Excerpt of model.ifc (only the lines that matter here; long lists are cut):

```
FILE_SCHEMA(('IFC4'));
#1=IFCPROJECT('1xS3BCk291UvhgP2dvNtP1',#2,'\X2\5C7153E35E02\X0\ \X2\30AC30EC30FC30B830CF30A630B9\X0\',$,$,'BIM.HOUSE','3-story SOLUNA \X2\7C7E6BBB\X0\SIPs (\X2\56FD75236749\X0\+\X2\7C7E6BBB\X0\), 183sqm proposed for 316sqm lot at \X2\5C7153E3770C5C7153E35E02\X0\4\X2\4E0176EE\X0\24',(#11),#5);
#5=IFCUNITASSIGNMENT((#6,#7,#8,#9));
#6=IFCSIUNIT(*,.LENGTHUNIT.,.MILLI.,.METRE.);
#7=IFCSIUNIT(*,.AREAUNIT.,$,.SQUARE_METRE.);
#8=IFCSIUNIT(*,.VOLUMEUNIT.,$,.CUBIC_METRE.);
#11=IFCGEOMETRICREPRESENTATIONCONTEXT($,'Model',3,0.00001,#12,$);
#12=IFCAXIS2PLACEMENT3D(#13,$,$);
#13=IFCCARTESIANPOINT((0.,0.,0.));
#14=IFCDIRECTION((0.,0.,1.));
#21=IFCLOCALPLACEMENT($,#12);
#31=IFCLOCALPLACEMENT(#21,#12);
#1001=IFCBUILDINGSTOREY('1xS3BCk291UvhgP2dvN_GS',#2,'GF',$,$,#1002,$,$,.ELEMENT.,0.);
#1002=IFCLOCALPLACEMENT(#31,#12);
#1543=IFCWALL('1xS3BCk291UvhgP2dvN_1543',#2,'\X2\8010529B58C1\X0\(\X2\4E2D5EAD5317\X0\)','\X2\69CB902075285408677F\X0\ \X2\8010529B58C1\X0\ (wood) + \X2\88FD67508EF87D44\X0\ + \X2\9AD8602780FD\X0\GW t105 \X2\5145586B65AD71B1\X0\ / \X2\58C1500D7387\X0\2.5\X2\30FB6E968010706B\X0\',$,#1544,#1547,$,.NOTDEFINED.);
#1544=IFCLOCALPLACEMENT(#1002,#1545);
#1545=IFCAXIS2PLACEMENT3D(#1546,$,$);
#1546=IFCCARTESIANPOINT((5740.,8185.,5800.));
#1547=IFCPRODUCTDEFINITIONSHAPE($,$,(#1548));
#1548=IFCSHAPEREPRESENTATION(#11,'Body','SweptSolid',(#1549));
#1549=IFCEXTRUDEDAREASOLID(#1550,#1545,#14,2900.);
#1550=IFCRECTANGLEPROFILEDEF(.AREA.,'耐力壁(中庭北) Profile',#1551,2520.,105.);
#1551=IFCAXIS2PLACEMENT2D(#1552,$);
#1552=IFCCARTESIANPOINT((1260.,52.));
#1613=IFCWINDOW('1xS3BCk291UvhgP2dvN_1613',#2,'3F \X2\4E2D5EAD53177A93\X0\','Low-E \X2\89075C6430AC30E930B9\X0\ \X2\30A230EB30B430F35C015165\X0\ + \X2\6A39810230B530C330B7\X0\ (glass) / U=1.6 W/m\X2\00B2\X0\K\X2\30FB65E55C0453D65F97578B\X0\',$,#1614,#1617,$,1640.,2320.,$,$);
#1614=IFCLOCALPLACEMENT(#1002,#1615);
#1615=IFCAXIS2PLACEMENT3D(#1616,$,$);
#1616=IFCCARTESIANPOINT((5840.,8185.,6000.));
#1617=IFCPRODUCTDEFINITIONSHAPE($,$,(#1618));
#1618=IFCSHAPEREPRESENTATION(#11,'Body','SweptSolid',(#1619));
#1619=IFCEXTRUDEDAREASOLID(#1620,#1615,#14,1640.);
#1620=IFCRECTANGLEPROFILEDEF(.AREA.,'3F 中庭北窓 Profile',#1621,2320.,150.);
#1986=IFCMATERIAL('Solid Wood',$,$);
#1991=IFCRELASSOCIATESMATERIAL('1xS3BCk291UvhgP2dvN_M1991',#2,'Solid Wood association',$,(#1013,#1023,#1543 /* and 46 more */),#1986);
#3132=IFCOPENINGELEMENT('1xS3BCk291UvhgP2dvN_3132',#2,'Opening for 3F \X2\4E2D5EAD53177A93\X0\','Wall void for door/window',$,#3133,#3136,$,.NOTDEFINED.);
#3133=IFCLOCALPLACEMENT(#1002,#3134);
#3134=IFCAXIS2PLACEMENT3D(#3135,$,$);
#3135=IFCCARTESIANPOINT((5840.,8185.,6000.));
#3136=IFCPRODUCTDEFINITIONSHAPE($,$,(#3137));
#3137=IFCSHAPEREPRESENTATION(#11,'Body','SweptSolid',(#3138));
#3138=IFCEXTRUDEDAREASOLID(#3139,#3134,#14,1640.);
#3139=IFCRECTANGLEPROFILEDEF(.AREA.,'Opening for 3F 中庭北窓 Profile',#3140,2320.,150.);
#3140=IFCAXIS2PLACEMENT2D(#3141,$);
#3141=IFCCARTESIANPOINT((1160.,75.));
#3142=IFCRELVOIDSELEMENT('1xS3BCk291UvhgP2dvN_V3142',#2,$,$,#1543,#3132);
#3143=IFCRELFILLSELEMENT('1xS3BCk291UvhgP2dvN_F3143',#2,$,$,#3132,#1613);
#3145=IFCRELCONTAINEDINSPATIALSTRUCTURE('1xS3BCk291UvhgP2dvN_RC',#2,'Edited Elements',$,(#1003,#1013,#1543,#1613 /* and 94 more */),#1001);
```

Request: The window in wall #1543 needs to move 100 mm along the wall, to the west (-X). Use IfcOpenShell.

```python
import ifcopenshell
import ifcopenshell.api.geometry
import ifcopenshell.util.placement
import ifcopenshell.util.unit

model = ifcopenshell.open("model.ifc")
unit_scale = ifcopenshell.util.unit.calculate_unit_scale(model)

window = model.by_id(1613)
opening = window.FillsVoids[0].RelatingOpeningElement
wall = opening.VoidsElements[0].RelatingBuildingElement

wall_matrix = ifcopenshell.util.placement.get_local_placement(wall.ObjectPlacement)
shift = wall_matrix[:3, 0] * -0.1 / unit_scale
before = ifcopenshell.util.placement.get_local_placement(window.ObjectPlacement)[:3, 3].copy()

# The window is not placed relative to its opening, so move both.
for product in (opening, window):
    matrix = ifcopenshell.util.placement.get_local_placement(product.ObjectPlacement)
    matrix[:3, 3] += shift
    ifcopenshell.api.geometry.edit_object_placement(model, product=product, matrix=matrix, is_si=False)

after = ifcopenshell.util.placement.get_local_placement(window.ObjectPlacement)[:3, 3]
print("window moved by", (after - before).round(3) + 0.0)

model.write("model_updated.ifc")
```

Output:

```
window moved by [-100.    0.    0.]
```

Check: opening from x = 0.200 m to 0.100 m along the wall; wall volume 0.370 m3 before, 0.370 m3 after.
